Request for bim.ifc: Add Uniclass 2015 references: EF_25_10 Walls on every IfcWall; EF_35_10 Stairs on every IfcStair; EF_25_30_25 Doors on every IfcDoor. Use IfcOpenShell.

First a look at what the model holds.

```python
import ifcopenshell

model = ifcopenshell.open("bim.ifc")
print(model.schema)
print("classifications:", [c.Name for c in model.by_type("IfcClassification")])
for ifc_class in ("IfcDoor", "IfcRoof", "IfcStair", "IfcWall", "IfcWindow"):
    print(ifc_class, len(model.by_type(ifc_class)))
```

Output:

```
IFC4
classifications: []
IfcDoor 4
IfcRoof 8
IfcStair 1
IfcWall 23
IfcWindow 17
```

```python
import ifcopenshell
import ifcopenshell.api.classification

model = ifcopenshell.open("bim.ifc")

system = ifcopenshell.api.classification.add_classification(model, classification="Uniclass 2015")

codes = {
    "IfcWall": ("EF_25_10", "Walls"),
    "IfcStair": ("EF_35_10", "Stairs"),
    "IfcDoor": ("EF_25_30_25", "Doors"),
}
for ifc_class, (code, name) in codes.items():
    products = model.by_type(ifc_class)
    ifcopenshell.api.classification.add_reference(
        model, products=products, classification=system, identification=code, name=name
    )
    print(code, len(products))

model.write("bim_updated.ifc")
```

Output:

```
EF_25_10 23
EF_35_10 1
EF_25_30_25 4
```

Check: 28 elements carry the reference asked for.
